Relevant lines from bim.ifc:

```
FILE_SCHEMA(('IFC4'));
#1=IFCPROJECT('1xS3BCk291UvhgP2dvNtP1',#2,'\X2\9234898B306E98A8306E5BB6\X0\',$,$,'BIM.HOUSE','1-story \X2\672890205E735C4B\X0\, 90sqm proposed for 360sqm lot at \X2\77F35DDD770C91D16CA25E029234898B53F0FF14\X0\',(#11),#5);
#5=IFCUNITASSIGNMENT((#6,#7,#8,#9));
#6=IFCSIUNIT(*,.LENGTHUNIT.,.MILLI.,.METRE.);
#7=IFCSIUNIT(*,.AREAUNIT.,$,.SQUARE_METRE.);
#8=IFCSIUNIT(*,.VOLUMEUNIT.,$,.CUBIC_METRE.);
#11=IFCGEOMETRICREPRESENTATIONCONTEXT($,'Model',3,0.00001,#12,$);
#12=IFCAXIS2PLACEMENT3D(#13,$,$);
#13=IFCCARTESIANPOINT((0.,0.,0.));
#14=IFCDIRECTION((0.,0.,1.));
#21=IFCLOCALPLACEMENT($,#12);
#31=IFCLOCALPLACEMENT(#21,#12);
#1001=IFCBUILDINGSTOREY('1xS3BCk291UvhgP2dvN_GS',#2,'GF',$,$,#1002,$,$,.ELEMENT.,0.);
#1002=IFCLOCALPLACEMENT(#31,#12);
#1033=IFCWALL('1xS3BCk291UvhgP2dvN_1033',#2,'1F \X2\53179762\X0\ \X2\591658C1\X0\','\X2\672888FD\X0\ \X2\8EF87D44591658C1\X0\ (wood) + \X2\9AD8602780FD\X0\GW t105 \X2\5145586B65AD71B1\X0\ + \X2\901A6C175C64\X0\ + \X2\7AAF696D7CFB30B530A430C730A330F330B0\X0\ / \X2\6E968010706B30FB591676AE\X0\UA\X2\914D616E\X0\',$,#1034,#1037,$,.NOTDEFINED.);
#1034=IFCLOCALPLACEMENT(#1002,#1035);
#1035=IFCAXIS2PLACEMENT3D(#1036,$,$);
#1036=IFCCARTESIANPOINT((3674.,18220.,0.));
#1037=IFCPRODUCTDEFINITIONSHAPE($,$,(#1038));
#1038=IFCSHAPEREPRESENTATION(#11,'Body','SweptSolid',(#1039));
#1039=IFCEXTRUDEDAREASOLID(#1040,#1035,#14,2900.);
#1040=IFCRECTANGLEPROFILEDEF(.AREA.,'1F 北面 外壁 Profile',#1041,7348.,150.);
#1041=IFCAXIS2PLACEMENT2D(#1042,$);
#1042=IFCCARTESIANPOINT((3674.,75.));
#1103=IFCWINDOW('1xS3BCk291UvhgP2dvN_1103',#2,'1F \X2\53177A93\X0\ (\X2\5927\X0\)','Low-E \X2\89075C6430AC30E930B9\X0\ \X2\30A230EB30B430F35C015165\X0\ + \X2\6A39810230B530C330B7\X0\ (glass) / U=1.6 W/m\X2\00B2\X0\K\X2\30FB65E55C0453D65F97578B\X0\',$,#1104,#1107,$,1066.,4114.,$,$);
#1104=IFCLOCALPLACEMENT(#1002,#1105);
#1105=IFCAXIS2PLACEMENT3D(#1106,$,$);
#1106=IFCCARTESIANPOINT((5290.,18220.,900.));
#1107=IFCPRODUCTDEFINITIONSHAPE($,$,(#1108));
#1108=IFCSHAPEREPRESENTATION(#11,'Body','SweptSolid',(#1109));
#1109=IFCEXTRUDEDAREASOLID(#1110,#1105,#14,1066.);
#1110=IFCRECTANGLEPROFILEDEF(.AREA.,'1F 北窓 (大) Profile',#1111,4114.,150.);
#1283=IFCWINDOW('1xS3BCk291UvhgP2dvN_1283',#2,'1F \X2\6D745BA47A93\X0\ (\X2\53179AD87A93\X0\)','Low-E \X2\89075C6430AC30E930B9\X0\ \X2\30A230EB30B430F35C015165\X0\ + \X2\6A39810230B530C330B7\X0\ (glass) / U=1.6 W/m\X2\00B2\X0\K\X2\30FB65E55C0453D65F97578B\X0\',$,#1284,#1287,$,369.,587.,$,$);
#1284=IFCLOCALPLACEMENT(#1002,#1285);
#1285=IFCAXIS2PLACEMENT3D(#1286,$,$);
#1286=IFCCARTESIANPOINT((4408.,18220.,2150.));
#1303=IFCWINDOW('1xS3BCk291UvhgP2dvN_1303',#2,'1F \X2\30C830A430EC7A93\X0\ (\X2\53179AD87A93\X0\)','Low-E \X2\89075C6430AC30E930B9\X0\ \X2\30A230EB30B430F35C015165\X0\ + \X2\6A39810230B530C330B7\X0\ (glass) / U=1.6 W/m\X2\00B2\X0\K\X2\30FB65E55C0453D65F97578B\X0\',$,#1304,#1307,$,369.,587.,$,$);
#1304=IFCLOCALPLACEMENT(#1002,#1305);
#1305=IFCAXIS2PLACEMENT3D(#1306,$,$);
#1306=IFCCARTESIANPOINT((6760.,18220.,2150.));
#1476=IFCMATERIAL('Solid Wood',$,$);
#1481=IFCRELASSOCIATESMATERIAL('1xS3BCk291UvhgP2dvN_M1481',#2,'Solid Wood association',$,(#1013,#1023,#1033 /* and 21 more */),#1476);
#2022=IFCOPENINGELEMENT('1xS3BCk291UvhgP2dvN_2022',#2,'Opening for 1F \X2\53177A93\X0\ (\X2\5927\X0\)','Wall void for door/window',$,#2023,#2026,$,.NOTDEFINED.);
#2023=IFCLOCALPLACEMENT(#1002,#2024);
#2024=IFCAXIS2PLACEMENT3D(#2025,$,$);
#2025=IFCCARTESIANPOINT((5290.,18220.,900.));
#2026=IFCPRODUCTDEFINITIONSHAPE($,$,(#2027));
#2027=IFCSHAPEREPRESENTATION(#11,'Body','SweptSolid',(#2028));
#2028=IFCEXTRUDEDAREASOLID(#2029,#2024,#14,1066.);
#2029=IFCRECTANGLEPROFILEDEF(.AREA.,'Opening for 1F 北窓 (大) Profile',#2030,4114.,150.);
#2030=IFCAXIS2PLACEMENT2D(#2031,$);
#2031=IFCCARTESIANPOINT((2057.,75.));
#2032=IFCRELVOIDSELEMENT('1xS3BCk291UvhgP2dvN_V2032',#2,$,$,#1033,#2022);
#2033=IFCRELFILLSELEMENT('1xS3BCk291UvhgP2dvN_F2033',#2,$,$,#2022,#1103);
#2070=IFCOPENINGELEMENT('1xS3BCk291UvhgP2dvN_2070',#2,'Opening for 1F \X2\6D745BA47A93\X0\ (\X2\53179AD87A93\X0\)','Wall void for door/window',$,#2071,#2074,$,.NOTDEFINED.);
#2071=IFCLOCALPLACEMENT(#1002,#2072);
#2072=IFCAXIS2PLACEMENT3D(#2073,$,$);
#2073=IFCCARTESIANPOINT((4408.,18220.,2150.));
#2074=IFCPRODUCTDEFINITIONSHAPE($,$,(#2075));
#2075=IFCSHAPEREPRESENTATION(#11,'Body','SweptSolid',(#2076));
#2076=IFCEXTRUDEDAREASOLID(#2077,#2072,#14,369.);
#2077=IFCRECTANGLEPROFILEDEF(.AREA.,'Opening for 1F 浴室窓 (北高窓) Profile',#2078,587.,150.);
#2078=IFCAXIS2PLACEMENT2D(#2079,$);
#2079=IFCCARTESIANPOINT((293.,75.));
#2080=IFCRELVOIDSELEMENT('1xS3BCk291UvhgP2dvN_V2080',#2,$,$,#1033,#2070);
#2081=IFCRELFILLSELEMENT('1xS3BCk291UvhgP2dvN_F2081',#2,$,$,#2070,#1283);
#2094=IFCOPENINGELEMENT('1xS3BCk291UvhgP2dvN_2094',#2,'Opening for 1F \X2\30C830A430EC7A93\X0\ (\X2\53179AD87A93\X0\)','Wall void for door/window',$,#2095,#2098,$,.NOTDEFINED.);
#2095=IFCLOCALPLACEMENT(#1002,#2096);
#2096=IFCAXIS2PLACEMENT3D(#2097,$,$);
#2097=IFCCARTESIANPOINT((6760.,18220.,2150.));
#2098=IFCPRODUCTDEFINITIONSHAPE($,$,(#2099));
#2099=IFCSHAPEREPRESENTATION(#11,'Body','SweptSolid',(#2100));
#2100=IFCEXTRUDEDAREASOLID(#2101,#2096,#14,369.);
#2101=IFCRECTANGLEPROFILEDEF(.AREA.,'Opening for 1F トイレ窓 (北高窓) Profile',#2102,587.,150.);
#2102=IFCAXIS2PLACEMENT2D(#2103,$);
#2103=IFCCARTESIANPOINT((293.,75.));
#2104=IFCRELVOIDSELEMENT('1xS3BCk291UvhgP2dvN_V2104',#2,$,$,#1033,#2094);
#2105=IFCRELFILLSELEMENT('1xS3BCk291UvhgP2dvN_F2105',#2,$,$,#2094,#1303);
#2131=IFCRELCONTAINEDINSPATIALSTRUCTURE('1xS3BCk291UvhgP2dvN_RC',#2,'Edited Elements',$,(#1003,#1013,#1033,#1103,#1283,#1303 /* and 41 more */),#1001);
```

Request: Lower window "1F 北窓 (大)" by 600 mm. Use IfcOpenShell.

```python
import numpy as np
import ifcopenshell
import ifcopenshell.api.geometry
import ifcopenshell.util.placement
import ifcopenshell.util.unit

model = ifcopenshell.open("bim.ifc")
unit_scale = ifcopenshell.util.unit.calculate_unit_scale(model)

window = model.by_id(1103)
opening = window.FillsVoids[0].RelatingOpeningElement
dz = -0.6 / unit_scale

shift = np.array([0.0, 0.0, dz])
# The window is not placed relative to its opening, so move both.
for product in (opening, window):
    matrix = ifcopenshell.util.placement.get_local_placement(product.ObjectPlacement)
    matrix[:3, 3] += shift
    ifcopenshell.api.geometry.edit_object_placement(model, product=product, matrix=matrix, is_si=False)

print(f"moved by {dz * unit_scale:+.3f} m")

model.write("bim_edited.ifc")
```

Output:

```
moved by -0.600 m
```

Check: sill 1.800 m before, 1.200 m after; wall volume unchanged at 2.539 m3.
